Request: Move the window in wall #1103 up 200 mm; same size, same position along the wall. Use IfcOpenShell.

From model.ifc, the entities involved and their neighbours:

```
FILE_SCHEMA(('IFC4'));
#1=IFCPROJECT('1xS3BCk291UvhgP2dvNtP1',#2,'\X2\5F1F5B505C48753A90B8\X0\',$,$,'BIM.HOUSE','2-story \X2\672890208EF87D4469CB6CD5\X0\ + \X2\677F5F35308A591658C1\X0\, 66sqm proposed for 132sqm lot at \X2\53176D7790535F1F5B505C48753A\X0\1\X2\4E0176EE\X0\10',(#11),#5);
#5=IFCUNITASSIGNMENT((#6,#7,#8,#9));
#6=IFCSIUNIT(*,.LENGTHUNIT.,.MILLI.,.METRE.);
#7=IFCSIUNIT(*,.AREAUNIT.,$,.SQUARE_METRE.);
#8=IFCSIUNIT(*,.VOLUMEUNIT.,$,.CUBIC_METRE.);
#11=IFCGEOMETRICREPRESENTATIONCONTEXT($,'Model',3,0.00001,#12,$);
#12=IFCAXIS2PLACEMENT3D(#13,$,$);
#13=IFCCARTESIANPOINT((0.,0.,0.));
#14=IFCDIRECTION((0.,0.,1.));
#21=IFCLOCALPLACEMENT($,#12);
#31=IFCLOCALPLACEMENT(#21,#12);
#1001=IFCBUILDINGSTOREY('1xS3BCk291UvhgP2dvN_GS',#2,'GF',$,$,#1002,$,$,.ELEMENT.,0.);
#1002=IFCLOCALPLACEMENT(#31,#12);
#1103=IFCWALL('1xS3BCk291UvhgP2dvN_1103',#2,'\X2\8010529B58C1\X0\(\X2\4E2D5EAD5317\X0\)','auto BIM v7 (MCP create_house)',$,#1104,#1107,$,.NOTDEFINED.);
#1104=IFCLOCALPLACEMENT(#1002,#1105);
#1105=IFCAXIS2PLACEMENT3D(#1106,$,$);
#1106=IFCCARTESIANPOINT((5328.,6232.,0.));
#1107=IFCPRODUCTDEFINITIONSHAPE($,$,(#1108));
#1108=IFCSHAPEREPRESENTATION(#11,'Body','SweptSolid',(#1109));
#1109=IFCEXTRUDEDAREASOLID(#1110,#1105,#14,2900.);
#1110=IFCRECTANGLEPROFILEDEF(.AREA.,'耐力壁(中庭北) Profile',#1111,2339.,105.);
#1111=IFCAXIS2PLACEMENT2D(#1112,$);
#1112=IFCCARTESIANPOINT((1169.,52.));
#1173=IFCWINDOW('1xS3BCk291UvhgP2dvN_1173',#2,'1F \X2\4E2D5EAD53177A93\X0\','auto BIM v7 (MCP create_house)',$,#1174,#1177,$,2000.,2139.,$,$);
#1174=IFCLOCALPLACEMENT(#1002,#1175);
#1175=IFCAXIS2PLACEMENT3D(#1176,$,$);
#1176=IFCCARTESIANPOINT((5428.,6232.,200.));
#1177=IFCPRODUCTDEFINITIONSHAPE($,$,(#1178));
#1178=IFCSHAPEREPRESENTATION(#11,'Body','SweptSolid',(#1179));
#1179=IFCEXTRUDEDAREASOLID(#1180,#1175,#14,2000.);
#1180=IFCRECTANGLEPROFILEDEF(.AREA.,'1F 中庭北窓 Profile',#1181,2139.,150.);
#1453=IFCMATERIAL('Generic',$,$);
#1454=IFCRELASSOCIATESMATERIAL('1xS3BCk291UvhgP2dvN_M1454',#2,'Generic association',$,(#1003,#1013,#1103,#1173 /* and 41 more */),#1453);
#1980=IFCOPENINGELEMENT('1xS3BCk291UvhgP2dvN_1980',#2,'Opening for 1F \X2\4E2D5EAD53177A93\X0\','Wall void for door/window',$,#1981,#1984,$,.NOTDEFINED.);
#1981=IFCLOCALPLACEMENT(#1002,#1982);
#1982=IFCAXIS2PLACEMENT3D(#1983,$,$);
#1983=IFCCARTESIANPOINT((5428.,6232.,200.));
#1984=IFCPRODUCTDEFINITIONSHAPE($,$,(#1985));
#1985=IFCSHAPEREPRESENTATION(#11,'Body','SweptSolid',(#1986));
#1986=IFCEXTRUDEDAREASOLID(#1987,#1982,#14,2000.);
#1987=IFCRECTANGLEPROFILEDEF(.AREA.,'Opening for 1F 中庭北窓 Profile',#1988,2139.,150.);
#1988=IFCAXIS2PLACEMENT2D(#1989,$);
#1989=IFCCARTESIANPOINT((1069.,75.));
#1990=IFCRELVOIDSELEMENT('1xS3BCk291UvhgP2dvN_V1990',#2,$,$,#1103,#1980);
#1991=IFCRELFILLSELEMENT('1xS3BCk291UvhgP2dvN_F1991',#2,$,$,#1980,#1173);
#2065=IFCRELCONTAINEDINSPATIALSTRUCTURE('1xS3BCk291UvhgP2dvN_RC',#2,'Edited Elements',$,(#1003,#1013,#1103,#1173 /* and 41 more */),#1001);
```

```python
import numpy as np
import ifcopenshell
import ifcopenshell.api.geometry
import ifcopenshell.util.placement
import ifcopenshell.util.unit

model = ifcopenshell.open("model.ifc")
unit_scale = ifcopenshell.util.unit.calculate_unit_scale(model)

window = model.by_guid("1xS3BCk291UvhgP2dvN_1173")
opening = window.FillsVoids[0].RelatingOpeningElement
dz = 0.2 / unit_scale

shift = np.array([0.0, 0.0, dz])
# The window is not placed relative to its opening, so move both.
for product in (opening, window):
    matrix = ifcopenshell.util.placement.get_local_placement(product.ObjectPlacement)
    matrix[:3, 3] += shift
    ifcopenshell.api.geometry.edit_object_placement(model, product=product, matrix=matrix, is_si=False)

print(f"moved by {dz * unit_scale:+.3f} m")

model.write("model_v2.ifc")
```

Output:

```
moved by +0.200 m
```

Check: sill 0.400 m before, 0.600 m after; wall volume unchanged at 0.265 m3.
